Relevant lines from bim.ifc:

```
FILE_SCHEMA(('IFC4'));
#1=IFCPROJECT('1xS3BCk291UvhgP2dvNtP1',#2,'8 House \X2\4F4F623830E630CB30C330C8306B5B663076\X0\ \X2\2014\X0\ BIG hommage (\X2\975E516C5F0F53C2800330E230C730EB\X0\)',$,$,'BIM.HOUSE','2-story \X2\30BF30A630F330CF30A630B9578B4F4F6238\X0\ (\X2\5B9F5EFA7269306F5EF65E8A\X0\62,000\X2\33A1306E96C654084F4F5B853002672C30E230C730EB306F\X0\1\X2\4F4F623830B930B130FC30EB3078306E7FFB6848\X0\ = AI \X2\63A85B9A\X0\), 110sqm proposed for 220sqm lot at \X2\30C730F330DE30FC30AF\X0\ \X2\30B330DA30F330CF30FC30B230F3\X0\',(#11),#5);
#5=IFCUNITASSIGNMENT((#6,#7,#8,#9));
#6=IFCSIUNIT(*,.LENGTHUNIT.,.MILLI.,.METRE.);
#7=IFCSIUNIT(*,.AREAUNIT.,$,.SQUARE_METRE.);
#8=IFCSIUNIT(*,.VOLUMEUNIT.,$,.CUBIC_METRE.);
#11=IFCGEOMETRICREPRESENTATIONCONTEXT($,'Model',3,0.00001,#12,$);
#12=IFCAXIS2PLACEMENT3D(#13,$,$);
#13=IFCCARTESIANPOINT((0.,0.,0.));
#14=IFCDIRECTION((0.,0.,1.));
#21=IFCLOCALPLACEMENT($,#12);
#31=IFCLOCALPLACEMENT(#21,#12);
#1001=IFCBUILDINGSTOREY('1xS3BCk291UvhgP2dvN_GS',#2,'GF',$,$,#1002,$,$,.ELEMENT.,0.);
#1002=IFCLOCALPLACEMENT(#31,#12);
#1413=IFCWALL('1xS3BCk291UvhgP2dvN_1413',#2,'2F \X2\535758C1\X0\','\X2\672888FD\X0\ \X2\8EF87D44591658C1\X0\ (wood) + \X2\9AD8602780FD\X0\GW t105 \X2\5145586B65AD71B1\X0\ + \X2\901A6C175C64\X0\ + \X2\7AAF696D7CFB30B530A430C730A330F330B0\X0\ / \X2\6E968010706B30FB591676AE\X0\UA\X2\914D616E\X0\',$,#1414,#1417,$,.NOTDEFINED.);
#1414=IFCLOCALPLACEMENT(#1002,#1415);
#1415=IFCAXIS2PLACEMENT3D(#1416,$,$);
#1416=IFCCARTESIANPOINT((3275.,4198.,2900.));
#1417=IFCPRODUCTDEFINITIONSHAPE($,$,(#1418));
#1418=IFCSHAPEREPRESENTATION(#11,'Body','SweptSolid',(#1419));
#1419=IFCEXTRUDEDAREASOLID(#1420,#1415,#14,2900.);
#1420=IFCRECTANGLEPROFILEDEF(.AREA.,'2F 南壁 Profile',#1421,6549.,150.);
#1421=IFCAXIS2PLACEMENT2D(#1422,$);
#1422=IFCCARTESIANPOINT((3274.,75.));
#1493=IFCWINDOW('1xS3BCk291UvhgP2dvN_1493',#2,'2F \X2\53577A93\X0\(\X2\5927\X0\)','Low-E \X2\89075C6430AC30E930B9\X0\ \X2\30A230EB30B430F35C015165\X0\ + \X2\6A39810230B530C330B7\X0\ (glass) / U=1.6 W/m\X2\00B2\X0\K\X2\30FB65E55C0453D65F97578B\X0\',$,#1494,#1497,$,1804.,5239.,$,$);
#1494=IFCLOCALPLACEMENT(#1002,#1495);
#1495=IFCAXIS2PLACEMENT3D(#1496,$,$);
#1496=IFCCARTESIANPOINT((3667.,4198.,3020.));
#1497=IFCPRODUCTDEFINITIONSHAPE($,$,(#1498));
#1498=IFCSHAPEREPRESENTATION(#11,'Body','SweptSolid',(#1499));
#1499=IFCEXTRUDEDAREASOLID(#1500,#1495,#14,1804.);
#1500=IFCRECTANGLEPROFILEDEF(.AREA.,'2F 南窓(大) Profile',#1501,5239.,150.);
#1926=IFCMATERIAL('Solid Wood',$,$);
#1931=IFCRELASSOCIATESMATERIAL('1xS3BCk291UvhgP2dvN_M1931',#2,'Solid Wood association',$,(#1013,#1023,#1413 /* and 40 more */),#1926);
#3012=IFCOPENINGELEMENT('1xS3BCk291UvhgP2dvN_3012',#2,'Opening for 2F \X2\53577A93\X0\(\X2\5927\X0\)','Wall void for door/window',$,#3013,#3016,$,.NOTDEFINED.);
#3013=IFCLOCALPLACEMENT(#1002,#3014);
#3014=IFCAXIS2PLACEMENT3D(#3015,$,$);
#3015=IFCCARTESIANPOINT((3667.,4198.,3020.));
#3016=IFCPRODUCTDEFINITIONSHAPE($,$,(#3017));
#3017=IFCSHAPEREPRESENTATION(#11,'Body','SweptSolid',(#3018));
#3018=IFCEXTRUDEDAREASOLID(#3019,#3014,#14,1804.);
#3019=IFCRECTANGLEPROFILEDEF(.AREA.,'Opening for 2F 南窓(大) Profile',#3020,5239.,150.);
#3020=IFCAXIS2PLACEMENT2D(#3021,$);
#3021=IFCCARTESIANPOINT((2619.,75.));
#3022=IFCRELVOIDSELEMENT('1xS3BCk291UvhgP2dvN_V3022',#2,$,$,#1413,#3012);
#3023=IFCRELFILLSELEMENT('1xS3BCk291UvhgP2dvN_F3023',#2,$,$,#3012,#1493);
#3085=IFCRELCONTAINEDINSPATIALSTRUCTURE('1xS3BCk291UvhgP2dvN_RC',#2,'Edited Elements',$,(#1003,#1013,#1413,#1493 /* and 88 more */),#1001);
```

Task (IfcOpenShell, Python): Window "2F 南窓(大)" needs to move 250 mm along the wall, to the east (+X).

```python
import ifcopenshell
import ifcopenshell.api.geometry
import ifcopenshell.util.placement
import ifcopenshell.util.unit

model = ifcopenshell.open("bim.ifc")
unit_scale = ifcopenshell.util.unit.calculate_unit_scale(model)

window = model.by_guid("1xS3BCk291UvhgP2dvN_1493")
opening = window.FillsVoids[0].RelatingOpeningElement
wall = opening.VoidsElements[0].RelatingBuildingElement

wall_matrix = ifcopenshell.util.placement.get_local_placement(wall.ObjectPlacement)
shift = wall_matrix[:3, 0] * 0.25 / unit_scale
before = ifcopenshell.util.placement.get_local_placement(window.ObjectPlacement)[:3, 3].copy()

# The window is not placed relative to its opening, so move both.
for product in (opening, window):
    matrix = ifcopenshell.util.placement.get_local_placement(product.ObjectPlacement)
    matrix[:3, 3] += shift
    ifcopenshell.api.geometry.edit_object_placement(model, product=product, matrix=matrix, is_si=False)

after = ifcopenshell.util.placement.get_local_placement(window.ObjectPlacement)[:3, 3]
print("window moved by", (after - before).round(3) + 0.0)

model.write("bim_edited.ifc")
```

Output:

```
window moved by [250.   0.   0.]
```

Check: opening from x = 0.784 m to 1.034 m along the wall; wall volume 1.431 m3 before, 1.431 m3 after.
